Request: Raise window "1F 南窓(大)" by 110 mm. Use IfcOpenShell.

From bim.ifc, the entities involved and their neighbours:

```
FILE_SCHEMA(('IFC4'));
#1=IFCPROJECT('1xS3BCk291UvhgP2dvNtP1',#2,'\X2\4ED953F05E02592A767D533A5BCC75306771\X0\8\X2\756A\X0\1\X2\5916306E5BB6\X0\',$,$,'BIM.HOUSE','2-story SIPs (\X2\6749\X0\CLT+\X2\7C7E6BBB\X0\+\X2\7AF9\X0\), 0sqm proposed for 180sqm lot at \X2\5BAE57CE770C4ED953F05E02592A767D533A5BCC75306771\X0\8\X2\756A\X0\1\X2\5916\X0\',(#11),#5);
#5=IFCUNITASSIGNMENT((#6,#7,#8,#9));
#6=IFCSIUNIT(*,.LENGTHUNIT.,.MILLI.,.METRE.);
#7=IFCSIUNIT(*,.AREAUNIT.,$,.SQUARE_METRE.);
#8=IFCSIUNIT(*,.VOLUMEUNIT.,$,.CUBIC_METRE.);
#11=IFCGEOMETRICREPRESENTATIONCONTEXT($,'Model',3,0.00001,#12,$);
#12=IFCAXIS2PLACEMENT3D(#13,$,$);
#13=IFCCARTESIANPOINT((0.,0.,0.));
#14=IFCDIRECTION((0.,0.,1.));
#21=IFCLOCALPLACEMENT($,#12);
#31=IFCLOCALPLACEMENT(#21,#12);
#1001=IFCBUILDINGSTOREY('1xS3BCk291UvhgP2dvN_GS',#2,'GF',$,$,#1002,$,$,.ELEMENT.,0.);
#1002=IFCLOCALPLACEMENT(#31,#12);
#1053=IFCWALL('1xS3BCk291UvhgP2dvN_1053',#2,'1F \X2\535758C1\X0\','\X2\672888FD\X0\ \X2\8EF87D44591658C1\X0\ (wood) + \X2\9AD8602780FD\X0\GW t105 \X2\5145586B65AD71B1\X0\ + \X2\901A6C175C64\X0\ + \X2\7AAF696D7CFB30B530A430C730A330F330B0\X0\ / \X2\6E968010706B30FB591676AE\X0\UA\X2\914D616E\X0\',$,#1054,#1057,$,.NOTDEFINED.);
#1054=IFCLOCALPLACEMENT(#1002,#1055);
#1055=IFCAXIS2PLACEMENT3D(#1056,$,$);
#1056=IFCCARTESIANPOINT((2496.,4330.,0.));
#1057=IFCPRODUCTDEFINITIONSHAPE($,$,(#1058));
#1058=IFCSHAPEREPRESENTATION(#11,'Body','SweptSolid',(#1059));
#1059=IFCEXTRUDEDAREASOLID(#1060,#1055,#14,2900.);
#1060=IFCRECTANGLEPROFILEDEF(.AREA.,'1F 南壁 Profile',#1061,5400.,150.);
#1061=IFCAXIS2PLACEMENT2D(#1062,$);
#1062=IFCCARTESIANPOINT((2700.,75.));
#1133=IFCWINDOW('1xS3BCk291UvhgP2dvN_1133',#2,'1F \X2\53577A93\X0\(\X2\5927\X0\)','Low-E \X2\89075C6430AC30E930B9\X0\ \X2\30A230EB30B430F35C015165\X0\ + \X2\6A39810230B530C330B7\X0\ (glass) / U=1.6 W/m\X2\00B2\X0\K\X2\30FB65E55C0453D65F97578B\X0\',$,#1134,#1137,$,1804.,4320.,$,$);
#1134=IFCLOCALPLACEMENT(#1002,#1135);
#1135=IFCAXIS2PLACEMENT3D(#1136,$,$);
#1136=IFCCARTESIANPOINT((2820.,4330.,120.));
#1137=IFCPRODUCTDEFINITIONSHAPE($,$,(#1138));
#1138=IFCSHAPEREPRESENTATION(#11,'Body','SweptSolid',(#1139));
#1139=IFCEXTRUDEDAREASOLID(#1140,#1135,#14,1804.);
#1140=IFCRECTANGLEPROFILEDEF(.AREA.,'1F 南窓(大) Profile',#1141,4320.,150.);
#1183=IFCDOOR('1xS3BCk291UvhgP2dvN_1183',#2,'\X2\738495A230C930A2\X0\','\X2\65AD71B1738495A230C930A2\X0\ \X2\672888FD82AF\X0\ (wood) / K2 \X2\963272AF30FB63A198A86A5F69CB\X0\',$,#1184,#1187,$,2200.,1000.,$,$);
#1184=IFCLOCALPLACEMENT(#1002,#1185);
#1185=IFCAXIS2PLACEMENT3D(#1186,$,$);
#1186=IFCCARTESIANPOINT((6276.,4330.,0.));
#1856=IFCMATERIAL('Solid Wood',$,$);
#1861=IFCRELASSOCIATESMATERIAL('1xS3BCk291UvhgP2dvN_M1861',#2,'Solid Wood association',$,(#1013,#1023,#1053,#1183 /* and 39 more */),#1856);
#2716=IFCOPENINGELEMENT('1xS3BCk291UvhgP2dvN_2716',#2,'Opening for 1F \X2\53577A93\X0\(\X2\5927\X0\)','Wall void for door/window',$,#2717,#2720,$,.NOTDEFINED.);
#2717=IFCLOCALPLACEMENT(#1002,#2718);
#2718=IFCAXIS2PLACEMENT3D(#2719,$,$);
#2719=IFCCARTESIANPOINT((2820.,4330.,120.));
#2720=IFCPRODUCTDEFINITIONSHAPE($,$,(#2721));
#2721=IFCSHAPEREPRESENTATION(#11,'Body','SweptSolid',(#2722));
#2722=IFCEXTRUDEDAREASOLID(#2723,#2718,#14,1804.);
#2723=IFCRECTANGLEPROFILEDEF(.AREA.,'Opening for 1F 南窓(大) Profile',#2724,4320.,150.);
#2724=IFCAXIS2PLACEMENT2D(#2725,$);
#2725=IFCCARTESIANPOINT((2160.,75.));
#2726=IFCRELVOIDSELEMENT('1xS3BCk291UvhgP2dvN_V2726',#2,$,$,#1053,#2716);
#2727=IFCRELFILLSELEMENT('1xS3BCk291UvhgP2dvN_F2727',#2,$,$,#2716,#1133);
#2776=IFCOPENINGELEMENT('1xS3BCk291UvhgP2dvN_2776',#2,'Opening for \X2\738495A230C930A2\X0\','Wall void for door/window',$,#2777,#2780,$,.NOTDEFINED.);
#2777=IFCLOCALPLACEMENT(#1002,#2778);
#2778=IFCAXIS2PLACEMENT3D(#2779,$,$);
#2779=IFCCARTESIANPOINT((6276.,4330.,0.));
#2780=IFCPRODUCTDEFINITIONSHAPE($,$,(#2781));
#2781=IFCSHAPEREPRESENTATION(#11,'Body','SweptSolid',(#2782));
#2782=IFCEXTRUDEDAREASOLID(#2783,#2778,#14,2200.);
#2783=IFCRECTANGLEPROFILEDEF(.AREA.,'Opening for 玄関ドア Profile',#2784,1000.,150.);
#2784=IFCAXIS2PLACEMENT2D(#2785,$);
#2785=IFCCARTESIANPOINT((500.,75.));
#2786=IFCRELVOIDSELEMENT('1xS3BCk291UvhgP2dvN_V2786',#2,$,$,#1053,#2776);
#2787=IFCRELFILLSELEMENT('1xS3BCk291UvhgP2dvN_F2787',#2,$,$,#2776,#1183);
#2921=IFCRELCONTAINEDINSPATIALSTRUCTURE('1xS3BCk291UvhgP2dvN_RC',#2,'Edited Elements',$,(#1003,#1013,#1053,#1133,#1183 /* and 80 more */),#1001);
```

```python
import numpy as np
import ifcopenshell
import ifcopenshell.api.geometry
import ifcopenshell.util.placement
import ifcopenshell.util.unit

model = ifcopenshell.open("bim.ifc")
unit_scale = ifcopenshell.util.unit.calculate_unit_scale(model)

window = model.by_guid("1xS3BCk291UvhgP2dvN_1133")
opening = window.FillsVoids[0].RelatingOpeningElement
dz = 110.0

shift = np.array([0.0, 0.0, dz])
# The window is not placed relative to its opening, so move both.
for product in (opening, window):
    matrix = ifcopenshell.util.placement.get_local_placement(product.ObjectPlacement)
    matrix[:3, 3] += shift
    ifcopenshell.api.geometry.edit_object_placement(model, product=product, matrix=matrix, is_si=False)

print(f"moved by {dz * unit_scale:+.3f} m")

model.write("bim-out.ifc")
```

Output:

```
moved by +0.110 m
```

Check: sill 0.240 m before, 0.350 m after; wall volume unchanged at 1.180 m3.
